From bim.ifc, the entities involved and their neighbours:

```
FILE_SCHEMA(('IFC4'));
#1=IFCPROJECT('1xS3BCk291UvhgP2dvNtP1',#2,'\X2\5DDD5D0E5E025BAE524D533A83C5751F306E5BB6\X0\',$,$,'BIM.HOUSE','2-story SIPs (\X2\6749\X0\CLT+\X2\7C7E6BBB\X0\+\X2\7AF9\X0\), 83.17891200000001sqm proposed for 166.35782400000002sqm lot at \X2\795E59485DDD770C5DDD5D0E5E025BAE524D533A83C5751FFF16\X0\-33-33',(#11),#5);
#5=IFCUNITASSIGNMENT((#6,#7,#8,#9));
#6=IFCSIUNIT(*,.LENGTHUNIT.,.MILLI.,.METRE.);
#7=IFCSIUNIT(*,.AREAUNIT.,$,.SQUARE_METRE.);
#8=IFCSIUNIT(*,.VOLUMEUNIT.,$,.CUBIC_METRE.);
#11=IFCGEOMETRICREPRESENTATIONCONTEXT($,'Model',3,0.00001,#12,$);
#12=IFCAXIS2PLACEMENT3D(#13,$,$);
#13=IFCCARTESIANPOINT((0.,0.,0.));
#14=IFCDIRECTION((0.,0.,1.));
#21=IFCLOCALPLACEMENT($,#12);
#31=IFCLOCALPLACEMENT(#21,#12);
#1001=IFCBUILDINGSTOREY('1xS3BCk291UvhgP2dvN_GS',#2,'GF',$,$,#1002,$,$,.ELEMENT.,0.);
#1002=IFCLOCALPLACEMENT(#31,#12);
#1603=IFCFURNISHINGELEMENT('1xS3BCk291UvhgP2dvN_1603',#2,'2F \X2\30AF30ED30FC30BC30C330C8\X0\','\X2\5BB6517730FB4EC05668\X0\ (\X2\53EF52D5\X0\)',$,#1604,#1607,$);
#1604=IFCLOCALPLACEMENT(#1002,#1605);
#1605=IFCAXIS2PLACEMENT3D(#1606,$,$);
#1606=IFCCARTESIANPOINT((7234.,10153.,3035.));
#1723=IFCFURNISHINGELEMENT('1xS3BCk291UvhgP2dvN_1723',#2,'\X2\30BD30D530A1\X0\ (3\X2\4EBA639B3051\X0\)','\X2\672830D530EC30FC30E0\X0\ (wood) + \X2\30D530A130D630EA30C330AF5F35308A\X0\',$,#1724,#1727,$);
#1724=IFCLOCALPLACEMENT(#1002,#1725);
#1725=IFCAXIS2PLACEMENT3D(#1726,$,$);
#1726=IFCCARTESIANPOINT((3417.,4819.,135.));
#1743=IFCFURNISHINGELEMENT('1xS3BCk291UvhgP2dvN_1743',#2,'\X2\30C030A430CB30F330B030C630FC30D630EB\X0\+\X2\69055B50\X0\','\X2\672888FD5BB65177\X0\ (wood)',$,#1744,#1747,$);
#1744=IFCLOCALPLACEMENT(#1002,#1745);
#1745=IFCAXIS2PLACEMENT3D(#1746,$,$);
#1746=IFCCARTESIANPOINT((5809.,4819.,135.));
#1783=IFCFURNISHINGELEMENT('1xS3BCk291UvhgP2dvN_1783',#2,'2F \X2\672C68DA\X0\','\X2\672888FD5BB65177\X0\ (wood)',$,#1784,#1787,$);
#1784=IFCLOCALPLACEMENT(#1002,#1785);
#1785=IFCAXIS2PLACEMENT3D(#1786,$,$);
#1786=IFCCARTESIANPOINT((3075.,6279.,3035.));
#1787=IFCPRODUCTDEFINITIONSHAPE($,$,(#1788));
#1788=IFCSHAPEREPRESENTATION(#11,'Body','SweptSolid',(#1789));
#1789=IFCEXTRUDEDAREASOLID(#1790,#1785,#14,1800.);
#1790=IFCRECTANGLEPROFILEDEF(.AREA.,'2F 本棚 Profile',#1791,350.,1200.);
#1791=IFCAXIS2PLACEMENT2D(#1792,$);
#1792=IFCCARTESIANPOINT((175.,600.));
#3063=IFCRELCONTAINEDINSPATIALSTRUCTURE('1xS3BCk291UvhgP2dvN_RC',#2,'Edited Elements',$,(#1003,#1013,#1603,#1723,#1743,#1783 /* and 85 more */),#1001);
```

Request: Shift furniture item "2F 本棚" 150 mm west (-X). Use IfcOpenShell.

```python
import ifcopenshell
import ifcopenshell.api.geometry
import ifcopenshell.util.placement

model = ifcopenshell.open("bim.ifc")

item = model.by_id(1783)
matrix = ifcopenshell.util.placement.get_local_placement(item.ObjectPlacement)
matrix[0, 3] -= 150.0
ifcopenshell.api.geometry.edit_object_placement(model, product=item, matrix=matrix, is_si=False)

print(ifcopenshell.util.placement.get_local_placement(item.ObjectPlacement).round(3) + 0.0)

model.write("bim-out.ifc")
```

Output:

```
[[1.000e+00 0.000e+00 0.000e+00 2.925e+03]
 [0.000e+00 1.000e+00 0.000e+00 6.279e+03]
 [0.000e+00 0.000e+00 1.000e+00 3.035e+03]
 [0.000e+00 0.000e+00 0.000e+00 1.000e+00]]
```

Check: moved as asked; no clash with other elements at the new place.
